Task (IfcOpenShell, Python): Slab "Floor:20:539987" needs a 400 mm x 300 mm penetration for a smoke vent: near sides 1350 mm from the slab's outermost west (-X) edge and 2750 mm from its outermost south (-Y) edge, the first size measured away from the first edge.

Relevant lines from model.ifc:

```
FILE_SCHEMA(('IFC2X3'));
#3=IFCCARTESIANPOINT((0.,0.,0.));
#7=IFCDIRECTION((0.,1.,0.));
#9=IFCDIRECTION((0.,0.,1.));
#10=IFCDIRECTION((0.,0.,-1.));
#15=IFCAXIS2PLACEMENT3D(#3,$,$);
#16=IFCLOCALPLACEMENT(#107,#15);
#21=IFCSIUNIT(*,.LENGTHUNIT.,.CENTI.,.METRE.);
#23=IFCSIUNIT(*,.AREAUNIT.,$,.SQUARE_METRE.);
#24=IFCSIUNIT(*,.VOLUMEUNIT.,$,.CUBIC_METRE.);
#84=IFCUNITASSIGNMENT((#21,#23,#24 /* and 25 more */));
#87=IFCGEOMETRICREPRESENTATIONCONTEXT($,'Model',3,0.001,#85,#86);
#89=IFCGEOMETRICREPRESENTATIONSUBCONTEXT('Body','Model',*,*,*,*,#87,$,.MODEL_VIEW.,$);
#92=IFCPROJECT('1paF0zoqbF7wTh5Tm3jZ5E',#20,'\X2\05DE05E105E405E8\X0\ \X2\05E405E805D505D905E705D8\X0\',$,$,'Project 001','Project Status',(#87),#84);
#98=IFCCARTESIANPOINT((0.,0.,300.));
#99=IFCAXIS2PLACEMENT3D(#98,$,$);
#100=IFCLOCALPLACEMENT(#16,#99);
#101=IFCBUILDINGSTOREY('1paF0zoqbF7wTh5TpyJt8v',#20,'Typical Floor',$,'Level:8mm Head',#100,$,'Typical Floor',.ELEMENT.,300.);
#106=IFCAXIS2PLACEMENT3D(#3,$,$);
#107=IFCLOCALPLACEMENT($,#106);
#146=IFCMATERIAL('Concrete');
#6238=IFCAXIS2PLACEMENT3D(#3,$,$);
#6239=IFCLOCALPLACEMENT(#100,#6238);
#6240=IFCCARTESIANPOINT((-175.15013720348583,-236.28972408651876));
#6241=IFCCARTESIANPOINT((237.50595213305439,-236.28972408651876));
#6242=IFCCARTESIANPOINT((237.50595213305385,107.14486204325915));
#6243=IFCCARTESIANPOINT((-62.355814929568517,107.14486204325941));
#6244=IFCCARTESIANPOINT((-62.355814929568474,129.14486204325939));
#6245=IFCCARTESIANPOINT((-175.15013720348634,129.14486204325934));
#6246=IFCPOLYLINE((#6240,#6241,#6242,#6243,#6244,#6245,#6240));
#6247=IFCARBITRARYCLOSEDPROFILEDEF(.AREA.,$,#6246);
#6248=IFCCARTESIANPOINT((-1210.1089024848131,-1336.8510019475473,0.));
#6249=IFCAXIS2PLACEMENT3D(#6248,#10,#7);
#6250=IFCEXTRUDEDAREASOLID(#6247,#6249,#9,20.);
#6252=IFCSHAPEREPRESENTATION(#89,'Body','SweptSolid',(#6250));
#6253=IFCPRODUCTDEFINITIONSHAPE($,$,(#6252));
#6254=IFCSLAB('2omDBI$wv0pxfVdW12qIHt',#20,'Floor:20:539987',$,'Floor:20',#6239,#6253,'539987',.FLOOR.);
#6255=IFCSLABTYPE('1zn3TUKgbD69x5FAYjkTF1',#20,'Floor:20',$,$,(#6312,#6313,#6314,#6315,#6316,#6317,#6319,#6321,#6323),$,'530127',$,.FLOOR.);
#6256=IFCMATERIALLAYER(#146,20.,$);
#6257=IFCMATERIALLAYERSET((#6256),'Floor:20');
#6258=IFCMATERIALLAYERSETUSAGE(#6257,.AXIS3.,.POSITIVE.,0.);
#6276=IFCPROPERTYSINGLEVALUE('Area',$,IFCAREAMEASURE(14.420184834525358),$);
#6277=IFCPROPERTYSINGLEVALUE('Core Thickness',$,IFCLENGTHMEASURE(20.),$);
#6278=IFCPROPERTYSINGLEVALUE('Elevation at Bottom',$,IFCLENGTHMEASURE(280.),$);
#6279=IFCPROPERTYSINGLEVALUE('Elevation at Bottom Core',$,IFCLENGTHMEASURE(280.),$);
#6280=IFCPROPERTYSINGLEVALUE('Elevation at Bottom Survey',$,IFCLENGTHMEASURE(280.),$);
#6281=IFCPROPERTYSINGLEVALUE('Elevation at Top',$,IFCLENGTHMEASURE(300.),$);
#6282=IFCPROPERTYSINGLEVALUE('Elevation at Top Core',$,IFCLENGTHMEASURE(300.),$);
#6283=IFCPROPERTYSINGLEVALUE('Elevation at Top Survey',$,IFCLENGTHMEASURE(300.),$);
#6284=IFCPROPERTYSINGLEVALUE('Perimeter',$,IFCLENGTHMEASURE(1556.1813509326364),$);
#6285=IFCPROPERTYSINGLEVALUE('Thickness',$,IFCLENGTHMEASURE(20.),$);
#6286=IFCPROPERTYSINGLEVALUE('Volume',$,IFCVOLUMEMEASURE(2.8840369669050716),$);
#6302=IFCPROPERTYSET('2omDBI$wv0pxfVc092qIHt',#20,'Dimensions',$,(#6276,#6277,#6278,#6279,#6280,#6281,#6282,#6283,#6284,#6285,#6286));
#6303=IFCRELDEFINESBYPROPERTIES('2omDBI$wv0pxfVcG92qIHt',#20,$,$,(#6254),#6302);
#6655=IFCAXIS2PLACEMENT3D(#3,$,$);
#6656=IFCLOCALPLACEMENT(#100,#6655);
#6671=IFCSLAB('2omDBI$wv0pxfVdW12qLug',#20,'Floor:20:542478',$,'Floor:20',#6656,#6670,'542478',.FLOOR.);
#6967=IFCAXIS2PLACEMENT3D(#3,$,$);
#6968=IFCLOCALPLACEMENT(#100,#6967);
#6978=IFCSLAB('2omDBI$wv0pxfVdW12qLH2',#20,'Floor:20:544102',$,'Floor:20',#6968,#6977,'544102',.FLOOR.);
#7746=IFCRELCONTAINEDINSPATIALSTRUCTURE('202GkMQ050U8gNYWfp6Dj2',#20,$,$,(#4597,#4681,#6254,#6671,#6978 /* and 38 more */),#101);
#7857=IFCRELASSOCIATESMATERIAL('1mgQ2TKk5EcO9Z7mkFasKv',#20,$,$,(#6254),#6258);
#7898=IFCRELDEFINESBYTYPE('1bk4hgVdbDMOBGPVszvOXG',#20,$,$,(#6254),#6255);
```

```python
import numpy as np
import ifcopenshell
import ifcopenshell.api.feature
import ifcopenshell.api.geometry
import ifcopenshell.api.pset
import ifcopenshell.api.root
import ifcopenshell.geom
import ifcopenshell.util.element
import ifcopenshell.util.placement
import ifcopenshell.util.representation
import ifcopenshell.util.shape
import ifcopenshell.util.unit

model = ifcopenshell.open("model.ifc")
unit_scale = ifcopenshell.util.unit.calculate_unit_scale(model)
area_scale = ifcopenshell.util.unit.calculate_unit_scale(model, "AREAUNIT")
volume_scale = ifcopenshell.util.unit.calculate_unit_scale(model, "VOLUMEUNIT")
settings = ifcopenshell.geom.settings()


def volume(element):
    """Net volume in cubic metres, openings subtracted."""
    shape = ifcopenshell.geom.create_shape(settings, element)
    return ifcopenshell.util.shape.get_volume(shape.geometry)


slab = model.by_guid("2omDBI$wv0pxfVdW12qIHt")
before = volume(slab)

# Extent in the slab's own axes, in metres. The edges named are its -X and -Y sides.
slab_shape = ifcopenshell.geom.create_shape(settings, slab)
vertices = ifcopenshell.util.shape.get_vertices(slab_shape.geometry)
x_min, y_min, bottom = vertices.min(axis=0)
top = vertices[:, 2].max()

opening = ifcopenshell.api.root.create_entity(model, ifc_class="IfcOpeningElement", name="Smoke vent opening")
context = ifcopenshell.util.representation.get_context(model, "Model", "Body", "MODEL_VIEW")
width, depth = 0.4, 0.3
outline = [(0.0, 0.0), (width, 0.0), (width, depth), (0.0, depth), (0.0, 0.0)]
# Overshoot both faces by 50 mm so the cut is clean.
shape = ifcopenshell.api.geometry.add_slab_representation(
    model, context=context, depth=top - bottom + 0.1, polyline=outline
)
ifcopenshell.api.geometry.assign_representation(model, product=opening, representation=shape)

matrix = ifcopenshell.util.placement.get_local_placement(slab.ObjectPlacement)
matrix[:, 3] = matrix @ np.append(np.array([x_min + 1.35, y_min + 2.75, bottom - 0.05]) / unit_scale, 1.0)
ifcopenshell.api.geometry.edit_object_placement(model, product=opening, matrix=matrix, is_si=False)
ifcopenshell.api.feature.add_feature(model, feature=opening, element=slab)

after = volume(slab)

# Update the slab's stored quantities.
pset = model.by_id(ifcopenshell.util.element.get_pset(slab, "Dimensions", should_inherit=False)["id"])
ifcopenshell.api.pset.edit_pset(model, pset=pset, properties={
    "Area": model.create_entity("IfcAreaMeasure", after / (top - bottom) / area_scale),
    "Volume": model.create_entity("IfcVolumeMeasure", after / volume_scale),
})

print(f"slab volume {before:.3f} -> {after:.3f} m3")

model.write("model-out.ifc")
```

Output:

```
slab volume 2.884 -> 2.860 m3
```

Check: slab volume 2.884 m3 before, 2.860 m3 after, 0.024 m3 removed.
